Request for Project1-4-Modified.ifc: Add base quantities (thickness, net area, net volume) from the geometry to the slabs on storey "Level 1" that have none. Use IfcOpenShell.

First a look at what the model holds.

```python
import ifcopenshell
import ifcopenshell.util.element
import ifcopenshell.util.unit

model = ifcopenshell.open("Project1-4-Modified.ifc")
print(model.schema)
for unit_type in ("LENGTHUNIT", "AREAUNIT", "VOLUMEUNIT"):
    print(unit_type, ifcopenshell.util.unit.calculate_unit_scale(model, unit_type))
storey = next(s for s in model.by_type("IfcBuildingStorey") if s.Name == "Level 1")
slabs = [e for e in ifcopenshell.util.element.get_decomposition(storey) if e.is_a("IfcSlab")]
for e in sorted(slabs, key=lambda e: e.id()):
    print(e.id(), e.is_a(), e.Name, list(ifcopenshell.util.element.get_psets(e, qtos_only=True)), sep=" | ")
```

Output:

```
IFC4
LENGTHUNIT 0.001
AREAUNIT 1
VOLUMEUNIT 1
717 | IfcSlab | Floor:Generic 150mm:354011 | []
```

```python
import ifcopenshell
import ifcopenshell.api.pset
import ifcopenshell.geom
import ifcopenshell.util.element
import ifcopenshell.util.shape
import ifcopenshell.util.unit

model = ifcopenshell.open("Project1-4-Modified.ifc")
unit_scale = ifcopenshell.util.unit.calculate_unit_scale(model)
area_scale = ifcopenshell.util.unit.calculate_unit_scale(model, "AREAUNIT")
volume_scale = ifcopenshell.util.unit.calculate_unit_scale(model, "VOLUMEUNIT")
settings = ifcopenshell.geom.settings()

storey = next(s for s in model.by_type("IfcBuildingStorey") if s.Name == "Level 1")
slabs = [e for e in ifcopenshell.util.element.get_decomposition(storey) if e.is_a("IfcSlab")]

for e in sorted(slabs, key=lambda e: e.id()):
    if ifcopenshell.util.element.get_psets(e, qtos_only=True, should_inherit=False):
        continue
    # Geometry comes back in metres, in the element's own axes.
    shape = ifcopenshell.geom.create_shape(settings, e)
    values = {
        "Width": ifcopenshell.util.shape.get_z(shape.geometry) / unit_scale,
        "NetArea": ifcopenshell.util.shape.get_footprint_area(shape.geometry) / area_scale,
        "NetVolume": ifcopenshell.util.shape.get_volume(shape.geometry) / volume_scale,
    }
    qto = ifcopenshell.api.pset.add_qto(model, product=e, name="Qto_SlabBaseQuantities")
    ifcopenshell.api.pset.edit_qto(model, qto=qto, properties=values)
    print(e.id(), {k: round(v, 3) for k, v in values.items()})

model.write("Project1-4-Modified_updated.ifc")
```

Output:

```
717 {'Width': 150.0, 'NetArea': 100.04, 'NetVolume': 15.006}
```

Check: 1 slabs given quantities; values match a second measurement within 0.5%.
